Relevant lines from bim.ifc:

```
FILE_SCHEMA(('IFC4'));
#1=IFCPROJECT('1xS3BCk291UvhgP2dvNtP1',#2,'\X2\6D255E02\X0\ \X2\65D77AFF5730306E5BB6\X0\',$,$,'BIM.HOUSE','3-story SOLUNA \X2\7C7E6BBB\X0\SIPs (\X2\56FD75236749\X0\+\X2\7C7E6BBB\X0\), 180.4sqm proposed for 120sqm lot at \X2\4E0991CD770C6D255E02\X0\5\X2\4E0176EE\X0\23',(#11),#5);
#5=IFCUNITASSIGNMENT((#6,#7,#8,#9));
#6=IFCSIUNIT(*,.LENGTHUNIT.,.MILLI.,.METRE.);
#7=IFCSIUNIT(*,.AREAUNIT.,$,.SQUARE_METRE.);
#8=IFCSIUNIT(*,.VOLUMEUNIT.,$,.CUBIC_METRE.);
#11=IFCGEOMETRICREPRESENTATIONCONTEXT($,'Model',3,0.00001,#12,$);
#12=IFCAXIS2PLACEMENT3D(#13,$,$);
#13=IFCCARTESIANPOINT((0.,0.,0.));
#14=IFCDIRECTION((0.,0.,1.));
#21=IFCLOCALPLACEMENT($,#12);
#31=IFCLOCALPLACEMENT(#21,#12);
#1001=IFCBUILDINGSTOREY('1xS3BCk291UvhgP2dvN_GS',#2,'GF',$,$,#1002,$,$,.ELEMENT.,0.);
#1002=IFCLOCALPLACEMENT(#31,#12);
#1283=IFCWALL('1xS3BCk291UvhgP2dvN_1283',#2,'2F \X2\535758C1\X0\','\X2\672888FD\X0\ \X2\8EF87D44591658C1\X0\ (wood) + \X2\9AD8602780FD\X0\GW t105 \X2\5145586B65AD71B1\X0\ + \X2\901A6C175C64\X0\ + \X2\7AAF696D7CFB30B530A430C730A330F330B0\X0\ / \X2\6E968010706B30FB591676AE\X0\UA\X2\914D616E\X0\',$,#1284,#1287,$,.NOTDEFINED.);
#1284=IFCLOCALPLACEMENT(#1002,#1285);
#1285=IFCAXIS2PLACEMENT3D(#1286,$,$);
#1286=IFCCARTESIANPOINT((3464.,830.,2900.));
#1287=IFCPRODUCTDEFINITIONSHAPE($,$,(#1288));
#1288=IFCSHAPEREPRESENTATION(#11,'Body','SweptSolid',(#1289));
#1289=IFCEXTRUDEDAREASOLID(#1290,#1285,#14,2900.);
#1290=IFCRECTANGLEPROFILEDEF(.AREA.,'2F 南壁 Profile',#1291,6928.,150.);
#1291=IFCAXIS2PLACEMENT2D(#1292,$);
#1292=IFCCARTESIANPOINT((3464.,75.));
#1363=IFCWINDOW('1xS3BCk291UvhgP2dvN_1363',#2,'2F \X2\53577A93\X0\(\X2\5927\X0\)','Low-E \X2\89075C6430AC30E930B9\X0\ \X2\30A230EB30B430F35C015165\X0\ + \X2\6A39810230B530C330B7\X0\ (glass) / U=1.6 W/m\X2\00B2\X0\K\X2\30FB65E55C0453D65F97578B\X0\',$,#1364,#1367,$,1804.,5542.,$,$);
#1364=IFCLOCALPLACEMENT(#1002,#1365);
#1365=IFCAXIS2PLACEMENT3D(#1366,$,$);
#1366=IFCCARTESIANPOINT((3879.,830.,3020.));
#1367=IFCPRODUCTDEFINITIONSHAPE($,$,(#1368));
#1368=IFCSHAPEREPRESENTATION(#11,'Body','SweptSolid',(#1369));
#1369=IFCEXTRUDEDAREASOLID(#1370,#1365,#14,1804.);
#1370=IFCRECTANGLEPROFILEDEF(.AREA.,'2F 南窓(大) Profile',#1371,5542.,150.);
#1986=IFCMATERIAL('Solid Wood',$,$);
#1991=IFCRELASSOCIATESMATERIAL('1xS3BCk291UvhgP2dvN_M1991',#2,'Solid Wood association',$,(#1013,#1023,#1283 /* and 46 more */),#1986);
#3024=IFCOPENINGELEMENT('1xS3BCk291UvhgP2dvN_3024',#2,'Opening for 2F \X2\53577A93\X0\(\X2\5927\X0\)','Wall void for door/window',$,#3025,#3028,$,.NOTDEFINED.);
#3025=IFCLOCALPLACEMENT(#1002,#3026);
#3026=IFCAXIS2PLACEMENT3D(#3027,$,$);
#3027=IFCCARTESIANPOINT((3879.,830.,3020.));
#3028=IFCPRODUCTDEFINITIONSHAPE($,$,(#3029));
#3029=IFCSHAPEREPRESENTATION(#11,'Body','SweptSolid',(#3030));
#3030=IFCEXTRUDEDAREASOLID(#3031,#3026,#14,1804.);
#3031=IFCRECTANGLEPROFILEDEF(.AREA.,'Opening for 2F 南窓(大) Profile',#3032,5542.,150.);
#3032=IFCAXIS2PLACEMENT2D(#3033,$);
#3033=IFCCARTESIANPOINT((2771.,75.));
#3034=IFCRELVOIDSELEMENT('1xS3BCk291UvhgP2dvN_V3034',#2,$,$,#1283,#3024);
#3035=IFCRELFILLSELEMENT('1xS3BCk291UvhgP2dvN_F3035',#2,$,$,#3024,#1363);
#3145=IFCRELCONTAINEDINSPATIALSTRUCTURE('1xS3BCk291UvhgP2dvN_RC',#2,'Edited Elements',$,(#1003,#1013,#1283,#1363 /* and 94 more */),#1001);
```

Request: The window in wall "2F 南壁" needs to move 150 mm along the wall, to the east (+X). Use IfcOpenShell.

```python
import ifcopenshell
import ifcopenshell.api.geometry
import ifcopenshell.util.placement
import ifcopenshell.util.unit

model = ifcopenshell.open("bim.ifc")
unit_scale = ifcopenshell.util.unit.calculate_unit_scale(model)

window = model.by_guid("1xS3BCk291UvhgP2dvN_1363")
opening = window.FillsVoids[0].RelatingOpeningElement
wall = opening.VoidsElements[0].RelatingBuildingElement

wall_matrix = ifcopenshell.util.placement.get_local_placement(wall.ObjectPlacement)
shift = wall_matrix[:3, 0] * 0.15 / unit_scale
before = ifcopenshell.util.placement.get_local_placement(window.ObjectPlacement)[:3, 3].copy()

# The window is not placed relative to its opening, so move both.
for product in (opening, window):
    matrix = ifcopenshell.util.placement.get_local_placement(product.ObjectPlacement)
    matrix[:3, 3] += shift
    ifcopenshell.api.geometry.edit_object_placement(model, product=product, matrix=matrix, is_si=False)

after = ifcopenshell.util.placement.get_local_placement(window.ObjectPlacement)[:3, 3]
print("window moved by", (after - before).round(3) + 0.0)

model.write("bim_updated.ifc")
```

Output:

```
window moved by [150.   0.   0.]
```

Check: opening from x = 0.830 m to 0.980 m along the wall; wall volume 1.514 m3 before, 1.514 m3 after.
